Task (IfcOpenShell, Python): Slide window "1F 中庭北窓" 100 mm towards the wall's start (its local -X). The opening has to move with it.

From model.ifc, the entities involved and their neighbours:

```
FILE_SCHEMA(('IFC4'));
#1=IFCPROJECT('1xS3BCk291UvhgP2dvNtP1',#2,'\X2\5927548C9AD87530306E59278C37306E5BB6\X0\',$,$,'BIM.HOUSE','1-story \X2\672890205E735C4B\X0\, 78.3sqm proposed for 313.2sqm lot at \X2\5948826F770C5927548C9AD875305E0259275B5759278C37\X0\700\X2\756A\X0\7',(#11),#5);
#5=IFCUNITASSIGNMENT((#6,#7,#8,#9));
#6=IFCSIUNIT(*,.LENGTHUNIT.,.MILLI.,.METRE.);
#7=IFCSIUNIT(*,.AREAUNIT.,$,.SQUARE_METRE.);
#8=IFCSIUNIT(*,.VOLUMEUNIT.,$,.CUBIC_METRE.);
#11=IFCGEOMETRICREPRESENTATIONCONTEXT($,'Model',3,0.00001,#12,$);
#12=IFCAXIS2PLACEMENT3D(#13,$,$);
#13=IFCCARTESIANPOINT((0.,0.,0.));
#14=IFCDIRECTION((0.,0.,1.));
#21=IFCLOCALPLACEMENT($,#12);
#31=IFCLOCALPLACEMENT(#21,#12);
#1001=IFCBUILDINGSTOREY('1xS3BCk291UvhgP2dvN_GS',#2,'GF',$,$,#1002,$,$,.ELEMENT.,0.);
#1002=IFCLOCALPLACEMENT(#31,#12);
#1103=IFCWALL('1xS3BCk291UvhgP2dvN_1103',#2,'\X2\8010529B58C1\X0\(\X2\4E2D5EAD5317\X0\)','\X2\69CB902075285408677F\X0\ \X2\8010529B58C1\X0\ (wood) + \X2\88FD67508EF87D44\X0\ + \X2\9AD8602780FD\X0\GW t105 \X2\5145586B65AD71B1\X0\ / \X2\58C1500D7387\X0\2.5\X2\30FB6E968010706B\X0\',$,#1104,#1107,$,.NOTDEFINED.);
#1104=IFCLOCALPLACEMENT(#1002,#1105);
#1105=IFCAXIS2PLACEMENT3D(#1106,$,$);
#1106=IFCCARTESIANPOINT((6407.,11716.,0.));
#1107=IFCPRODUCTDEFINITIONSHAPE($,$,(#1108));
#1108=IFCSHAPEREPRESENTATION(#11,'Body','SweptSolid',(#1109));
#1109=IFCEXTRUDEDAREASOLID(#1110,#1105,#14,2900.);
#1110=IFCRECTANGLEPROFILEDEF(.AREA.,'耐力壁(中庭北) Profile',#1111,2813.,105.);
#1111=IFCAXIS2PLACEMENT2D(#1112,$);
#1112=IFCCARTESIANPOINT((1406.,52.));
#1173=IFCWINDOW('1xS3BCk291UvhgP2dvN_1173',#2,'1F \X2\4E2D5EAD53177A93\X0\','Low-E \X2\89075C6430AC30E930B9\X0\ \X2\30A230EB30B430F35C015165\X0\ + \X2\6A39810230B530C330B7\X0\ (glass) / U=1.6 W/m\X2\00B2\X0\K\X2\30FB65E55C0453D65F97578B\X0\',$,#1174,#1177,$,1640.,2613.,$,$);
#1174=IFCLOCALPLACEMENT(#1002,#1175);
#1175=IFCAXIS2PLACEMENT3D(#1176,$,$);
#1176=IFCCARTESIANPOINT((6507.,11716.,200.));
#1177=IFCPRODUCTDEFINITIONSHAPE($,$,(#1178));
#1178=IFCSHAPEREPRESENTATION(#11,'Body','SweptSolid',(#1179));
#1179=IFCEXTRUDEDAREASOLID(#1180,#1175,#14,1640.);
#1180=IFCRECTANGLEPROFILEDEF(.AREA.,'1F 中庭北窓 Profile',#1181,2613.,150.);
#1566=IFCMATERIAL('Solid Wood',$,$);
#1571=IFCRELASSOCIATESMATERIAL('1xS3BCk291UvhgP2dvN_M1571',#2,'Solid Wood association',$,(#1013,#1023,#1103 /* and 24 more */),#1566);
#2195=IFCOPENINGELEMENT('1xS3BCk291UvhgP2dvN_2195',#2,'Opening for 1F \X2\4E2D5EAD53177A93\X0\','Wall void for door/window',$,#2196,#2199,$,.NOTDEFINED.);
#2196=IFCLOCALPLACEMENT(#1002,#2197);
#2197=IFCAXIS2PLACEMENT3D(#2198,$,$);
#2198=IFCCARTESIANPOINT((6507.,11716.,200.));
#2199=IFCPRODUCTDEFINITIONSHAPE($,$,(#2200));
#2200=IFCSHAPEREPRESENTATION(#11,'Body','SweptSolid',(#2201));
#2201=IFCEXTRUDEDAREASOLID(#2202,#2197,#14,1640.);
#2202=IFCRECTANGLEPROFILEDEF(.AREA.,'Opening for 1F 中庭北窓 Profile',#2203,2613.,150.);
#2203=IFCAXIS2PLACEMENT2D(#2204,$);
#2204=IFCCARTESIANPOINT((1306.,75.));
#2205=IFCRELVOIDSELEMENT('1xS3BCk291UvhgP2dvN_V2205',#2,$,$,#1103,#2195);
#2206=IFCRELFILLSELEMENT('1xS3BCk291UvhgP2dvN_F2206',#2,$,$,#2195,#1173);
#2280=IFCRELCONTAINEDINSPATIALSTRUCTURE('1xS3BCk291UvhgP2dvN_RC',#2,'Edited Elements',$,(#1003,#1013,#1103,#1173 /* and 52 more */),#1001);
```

```python
import ifcopenshell
import ifcopenshell.api.geometry
import ifcopenshell.util.placement

model = ifcopenshell.open("model.ifc")

window = model.by_guid("1xS3BCk291UvhgP2dvN_1173")
opening = window.FillsVoids[0].RelatingOpeningElement
wall = opening.VoidsElements[0].RelatingBuildingElement

wall_matrix = ifcopenshell.util.placement.get_local_placement(wall.ObjectPlacement)
shift = wall_matrix[:3, 0] * -100.0
before = ifcopenshell.util.placement.get_local_placement(window.ObjectPlacement)[:3, 3].copy()

# The window is not placed relative to its opening, so move both.
for product in (opening, window):
    matrix = ifcopenshell.util.placement.get_local_placement(product.ObjectPlacement)
    matrix[:3, 3] += shift
    ifcopenshell.api.geometry.edit_object_placement(model, product=product, matrix=matrix, is_si=False)

after = ifcopenshell.util.placement.get_local_placement(window.ObjectPlacement)[:3, 3]
print("window moved by", (after - before).round(3) + 0.0)

model.write("model_rev.ifc")
```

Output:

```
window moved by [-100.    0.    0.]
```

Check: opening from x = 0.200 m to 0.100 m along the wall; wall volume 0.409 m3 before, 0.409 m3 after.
